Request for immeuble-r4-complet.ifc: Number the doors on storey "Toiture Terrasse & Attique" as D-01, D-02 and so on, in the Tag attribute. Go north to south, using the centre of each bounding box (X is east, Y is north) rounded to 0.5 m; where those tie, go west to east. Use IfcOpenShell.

First a look at what the model holds.

```python
import ifcopenshell
import ifcopenshell.util.element
import ifcopenshell.util.placement

model = ifcopenshell.open("immeuble-r4-complet.ifc")
print(model.schema)
storey = next(s for s in model.by_type("IfcBuildingStorey") if s.Name == "Toiture Terrasse & Attique")
doors = [e for e in ifcopenshell.util.element.get_decomposition(storey) if e.is_a("IfcDoor")]
for e in sorted(doors, key=lambda e: e.id()):
    origin = ifcopenshell.util.placement.get_local_placement(e.ObjectPlacement)[:3, 3]
    print(e.id(), e.Tag, e.Name, origin.round(2) + 0.0, sep=" | ")
```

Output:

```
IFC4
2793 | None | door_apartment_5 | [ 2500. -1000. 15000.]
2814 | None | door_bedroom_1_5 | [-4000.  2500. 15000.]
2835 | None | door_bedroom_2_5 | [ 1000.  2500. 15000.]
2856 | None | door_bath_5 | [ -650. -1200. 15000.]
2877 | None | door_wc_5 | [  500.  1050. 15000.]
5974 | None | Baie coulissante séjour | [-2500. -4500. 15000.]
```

```python
import ifcopenshell
import ifcopenshell.geom
import ifcopenshell.util.element
import ifcopenshell.util.shape

model = ifcopenshell.open("immeuble-r4-complet.ifc")
settings = ifcopenshell.geom.settings()
settings.set("use-world-coords", True)


def centre(element):
    shape = ifcopenshell.geom.create_shape(settings, element)
    return ifcopenshell.util.shape.get_bbox_centroid(shape.geometry)


storey = next(s for s in model.by_type("IfcBuildingStorey") if s.Name == "Toiture Terrasse & Attique")
doors = [e for e in ifcopenshell.util.element.get_decomposition(storey) if e.is_a("IfcDoor")]

# Insertion points can sit at a corner or the storey origin, so sort by the geometry (in metres).
centres = {e: centre(e) for e in doors}
doors.sort(key=lambda e: (-round(centres[e][1] / 0.5), centres[e][0]))

for i, e in enumerate(doors, start=1):
    number = f"D-{i:02d}"
    e.Tag = number
    print(e.id(), number)

model.write("immeuble-r4-complet_edited.ifc")
```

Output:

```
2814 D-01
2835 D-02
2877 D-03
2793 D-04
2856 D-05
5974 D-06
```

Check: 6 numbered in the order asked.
